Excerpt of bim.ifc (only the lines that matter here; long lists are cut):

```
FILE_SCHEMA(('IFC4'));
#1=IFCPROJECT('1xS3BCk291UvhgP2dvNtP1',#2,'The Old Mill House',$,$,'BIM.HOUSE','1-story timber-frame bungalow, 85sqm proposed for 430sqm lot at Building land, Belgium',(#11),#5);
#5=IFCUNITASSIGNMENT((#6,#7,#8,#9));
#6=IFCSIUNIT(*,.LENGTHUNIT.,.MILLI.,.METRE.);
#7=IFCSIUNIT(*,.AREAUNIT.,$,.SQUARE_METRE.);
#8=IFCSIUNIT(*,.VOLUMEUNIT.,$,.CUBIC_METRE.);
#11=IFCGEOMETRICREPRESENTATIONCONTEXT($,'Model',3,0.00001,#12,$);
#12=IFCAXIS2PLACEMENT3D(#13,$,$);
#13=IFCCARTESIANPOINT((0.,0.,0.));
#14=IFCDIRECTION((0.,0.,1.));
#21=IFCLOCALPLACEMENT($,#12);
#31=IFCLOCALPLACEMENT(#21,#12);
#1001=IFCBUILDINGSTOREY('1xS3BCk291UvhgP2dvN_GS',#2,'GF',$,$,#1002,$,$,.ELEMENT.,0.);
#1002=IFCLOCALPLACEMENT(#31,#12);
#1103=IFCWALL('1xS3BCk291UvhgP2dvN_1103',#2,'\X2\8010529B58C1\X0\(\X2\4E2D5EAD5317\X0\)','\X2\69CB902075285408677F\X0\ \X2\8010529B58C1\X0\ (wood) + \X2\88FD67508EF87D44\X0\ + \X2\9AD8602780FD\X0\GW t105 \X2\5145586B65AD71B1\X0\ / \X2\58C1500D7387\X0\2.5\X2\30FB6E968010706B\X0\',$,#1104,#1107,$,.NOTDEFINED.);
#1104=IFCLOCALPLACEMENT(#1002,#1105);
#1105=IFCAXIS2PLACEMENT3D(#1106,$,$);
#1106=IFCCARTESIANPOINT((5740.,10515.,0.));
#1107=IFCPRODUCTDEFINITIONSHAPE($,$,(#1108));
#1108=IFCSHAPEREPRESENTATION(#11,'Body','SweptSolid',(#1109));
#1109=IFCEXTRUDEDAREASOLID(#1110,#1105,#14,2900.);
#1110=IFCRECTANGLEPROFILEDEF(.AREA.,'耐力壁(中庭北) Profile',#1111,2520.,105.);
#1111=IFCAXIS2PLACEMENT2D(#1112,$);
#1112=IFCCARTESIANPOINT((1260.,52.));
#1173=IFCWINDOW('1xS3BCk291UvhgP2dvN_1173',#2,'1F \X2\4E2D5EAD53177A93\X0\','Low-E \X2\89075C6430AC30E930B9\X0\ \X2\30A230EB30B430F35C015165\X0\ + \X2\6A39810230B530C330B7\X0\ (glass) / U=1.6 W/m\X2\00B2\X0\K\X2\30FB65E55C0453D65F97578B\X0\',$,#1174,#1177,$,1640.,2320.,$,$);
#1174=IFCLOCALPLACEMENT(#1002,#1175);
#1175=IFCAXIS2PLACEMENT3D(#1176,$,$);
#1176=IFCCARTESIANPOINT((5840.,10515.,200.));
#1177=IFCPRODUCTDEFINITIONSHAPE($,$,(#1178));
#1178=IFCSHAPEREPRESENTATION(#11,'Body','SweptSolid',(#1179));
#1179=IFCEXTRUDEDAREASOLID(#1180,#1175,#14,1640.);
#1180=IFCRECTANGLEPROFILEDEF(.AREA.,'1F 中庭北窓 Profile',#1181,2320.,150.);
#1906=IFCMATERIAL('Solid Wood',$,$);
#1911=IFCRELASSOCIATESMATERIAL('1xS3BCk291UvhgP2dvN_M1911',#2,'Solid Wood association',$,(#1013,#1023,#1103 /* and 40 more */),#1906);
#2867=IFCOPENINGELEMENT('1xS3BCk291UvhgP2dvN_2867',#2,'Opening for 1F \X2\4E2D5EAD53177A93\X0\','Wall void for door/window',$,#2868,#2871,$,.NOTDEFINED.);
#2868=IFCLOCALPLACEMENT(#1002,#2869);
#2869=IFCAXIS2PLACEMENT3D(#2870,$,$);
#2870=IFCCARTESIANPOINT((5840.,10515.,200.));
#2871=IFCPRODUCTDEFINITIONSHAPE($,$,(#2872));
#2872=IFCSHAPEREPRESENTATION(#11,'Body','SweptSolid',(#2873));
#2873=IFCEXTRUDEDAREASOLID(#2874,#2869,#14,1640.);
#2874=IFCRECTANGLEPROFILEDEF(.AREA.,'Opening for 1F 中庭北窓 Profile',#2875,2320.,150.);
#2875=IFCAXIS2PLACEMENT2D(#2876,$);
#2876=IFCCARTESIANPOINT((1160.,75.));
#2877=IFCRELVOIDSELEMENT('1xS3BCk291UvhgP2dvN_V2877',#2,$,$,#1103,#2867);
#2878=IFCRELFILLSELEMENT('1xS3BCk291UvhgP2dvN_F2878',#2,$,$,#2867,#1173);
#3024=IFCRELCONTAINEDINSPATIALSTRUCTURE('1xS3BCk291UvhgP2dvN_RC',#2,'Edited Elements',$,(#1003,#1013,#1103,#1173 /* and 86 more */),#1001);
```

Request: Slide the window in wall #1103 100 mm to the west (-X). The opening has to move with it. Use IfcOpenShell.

```python
import ifcopenshell
import ifcopenshell.api.geometry
import ifcopenshell.util.placement

model = ifcopenshell.open("bim.ifc")

window = model.by_guid("1xS3BCk291UvhgP2dvN_1173")
opening = window.FillsVoids[0].RelatingOpeningElement
wall = opening.VoidsElements[0].RelatingBuildingElement

wall_matrix = ifcopenshell.util.placement.get_local_placement(wall.ObjectPlacement)
shift = wall_matrix[:3, 0] * -100.0
before = ifcopenshell.util.placement.get_local_placement(window.ObjectPlacement)[:3, 3].copy()

# The window is not placed relative to its opening, so move both.
for product in (opening, window):
    matrix = ifcopenshell.util.placement.get_local_placement(product.ObjectPlacement)
    matrix[:3, 3] += shift
    ifcopenshell.api.geometry.edit_object_placement(model, product=product, matrix=matrix, is_si=False)

after = ifcopenshell.util.placement.get_local_placement(window.ObjectPlacement)[:3, 3]
print("window moved by", (after - before).round(3) + 0.0)

model.write("bim_updated.ifc")
```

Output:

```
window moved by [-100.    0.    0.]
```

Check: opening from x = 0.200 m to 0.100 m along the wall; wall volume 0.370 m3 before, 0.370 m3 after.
